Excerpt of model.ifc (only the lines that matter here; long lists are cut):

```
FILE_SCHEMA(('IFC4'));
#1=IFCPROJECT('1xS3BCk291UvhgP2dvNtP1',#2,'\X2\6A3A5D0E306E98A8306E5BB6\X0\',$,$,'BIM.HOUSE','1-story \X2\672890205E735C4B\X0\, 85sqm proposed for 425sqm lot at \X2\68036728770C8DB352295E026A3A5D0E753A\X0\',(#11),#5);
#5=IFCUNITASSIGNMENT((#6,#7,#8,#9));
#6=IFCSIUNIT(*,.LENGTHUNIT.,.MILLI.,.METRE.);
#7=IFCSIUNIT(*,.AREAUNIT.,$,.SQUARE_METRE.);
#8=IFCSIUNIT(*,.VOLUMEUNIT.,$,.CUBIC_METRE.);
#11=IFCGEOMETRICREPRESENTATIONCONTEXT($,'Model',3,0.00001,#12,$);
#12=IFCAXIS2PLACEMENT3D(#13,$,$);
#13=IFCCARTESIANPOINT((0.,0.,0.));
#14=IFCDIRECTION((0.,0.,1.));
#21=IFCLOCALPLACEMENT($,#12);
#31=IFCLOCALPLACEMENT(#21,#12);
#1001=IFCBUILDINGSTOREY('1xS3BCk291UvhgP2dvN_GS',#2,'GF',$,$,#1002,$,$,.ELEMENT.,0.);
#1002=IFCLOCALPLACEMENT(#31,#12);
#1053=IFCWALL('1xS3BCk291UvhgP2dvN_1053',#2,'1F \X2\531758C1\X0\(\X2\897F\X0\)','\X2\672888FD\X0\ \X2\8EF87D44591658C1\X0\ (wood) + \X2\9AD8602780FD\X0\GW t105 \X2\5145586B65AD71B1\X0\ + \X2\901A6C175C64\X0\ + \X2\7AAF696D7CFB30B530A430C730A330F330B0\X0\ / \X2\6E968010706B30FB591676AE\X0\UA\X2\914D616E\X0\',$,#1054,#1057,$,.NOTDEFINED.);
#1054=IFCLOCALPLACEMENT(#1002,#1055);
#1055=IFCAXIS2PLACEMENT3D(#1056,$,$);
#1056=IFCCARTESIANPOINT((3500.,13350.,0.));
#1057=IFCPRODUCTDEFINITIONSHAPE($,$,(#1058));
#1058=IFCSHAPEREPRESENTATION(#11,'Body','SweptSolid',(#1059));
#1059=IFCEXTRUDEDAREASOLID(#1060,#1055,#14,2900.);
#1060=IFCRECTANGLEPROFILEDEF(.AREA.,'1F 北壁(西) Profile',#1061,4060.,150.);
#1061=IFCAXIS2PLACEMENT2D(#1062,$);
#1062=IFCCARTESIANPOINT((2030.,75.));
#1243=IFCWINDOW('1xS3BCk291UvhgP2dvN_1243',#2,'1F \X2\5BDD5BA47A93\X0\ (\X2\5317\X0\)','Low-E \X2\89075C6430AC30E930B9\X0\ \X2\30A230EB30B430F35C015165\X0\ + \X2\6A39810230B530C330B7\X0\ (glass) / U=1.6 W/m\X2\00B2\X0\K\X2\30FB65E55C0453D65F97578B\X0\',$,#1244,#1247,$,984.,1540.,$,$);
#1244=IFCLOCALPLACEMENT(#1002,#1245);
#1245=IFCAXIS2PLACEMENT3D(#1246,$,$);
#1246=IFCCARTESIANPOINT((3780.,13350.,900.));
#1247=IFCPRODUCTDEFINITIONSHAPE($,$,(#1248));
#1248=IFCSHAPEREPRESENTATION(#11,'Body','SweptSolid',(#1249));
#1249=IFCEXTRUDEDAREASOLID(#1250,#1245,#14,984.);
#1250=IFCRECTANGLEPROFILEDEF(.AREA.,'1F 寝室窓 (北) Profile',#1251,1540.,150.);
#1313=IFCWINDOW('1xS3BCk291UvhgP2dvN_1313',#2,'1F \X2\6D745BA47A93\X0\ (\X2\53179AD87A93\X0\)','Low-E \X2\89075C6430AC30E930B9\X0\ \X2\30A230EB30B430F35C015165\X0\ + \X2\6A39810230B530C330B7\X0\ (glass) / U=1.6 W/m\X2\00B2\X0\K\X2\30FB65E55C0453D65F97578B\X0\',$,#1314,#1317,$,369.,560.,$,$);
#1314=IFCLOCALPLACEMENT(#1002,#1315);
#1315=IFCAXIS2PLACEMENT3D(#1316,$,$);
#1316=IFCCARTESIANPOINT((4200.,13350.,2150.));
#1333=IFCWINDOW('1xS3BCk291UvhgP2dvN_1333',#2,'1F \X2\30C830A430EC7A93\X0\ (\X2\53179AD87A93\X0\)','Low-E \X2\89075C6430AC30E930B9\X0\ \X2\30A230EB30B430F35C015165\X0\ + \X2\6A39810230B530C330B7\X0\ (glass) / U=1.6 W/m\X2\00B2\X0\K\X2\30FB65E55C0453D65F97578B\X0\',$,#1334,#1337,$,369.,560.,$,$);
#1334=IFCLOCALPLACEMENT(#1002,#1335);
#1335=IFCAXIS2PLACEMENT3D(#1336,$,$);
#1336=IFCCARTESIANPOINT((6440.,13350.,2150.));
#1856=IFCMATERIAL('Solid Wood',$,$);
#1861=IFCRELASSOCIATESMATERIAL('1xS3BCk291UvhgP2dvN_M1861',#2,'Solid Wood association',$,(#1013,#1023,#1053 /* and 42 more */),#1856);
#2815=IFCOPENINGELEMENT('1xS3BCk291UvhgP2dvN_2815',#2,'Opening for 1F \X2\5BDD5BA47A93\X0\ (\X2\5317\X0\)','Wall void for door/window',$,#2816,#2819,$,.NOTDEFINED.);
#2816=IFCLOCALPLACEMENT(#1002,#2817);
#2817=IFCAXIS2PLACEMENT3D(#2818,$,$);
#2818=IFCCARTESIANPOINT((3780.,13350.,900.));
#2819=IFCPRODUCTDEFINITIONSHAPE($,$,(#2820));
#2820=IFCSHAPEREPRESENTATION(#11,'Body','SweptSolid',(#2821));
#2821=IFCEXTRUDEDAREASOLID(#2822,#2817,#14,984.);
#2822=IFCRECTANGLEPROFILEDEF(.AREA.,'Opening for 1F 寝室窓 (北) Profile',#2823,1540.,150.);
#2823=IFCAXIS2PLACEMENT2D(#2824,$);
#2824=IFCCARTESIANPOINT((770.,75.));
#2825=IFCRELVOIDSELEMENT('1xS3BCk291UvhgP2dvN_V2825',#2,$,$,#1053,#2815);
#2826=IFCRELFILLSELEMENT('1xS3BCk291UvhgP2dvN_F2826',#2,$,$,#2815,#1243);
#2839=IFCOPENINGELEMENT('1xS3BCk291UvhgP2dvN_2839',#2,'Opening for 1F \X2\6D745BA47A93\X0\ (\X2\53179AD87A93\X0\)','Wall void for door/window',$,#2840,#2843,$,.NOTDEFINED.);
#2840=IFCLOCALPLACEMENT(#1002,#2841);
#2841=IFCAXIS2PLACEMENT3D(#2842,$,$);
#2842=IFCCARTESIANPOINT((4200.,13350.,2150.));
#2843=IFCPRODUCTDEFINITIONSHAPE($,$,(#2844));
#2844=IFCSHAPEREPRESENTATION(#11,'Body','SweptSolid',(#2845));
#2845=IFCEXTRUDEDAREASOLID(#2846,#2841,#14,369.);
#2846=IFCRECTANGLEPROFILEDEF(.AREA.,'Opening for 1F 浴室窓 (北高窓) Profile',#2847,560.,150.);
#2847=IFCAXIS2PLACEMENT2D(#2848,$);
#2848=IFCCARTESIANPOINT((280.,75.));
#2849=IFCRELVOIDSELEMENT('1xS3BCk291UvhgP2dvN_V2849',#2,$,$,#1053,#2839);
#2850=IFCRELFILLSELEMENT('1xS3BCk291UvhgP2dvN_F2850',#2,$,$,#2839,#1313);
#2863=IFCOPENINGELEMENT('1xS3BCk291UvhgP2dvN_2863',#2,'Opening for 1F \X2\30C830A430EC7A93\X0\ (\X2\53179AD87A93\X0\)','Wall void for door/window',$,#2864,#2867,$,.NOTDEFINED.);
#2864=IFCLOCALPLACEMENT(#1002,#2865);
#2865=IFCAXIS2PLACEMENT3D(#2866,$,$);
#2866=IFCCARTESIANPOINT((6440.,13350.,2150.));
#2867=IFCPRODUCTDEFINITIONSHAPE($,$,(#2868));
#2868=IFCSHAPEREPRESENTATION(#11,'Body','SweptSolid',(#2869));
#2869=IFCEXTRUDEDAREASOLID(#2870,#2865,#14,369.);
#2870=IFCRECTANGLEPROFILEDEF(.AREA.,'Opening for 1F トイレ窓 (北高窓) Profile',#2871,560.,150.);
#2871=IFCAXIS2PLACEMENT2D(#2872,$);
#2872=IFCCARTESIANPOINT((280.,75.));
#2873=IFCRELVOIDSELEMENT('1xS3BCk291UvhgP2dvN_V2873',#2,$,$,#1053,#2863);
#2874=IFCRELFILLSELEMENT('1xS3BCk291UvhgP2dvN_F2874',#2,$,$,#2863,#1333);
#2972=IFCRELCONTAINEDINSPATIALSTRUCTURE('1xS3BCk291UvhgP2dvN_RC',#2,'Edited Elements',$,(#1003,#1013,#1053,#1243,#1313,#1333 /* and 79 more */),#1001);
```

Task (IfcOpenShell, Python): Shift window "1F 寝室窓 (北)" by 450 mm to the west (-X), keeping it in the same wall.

```python
import ifcopenshell
import ifcopenshell.api.geometry
import ifcopenshell.util.placement

model = ifcopenshell.open("model.ifc")

window = model.by_guid("1xS3BCk291UvhgP2dvN_1243")
opening = window.FillsVoids[0].RelatingOpeningElement
wall = opening.VoidsElements[0].RelatingBuildingElement

wall_matrix = ifcopenshell.util.placement.get_local_placement(wall.ObjectPlacement)
shift = wall_matrix[:3, 0] * -450.0
before = ifcopenshell.util.placement.get_local_placement(window.ObjectPlacement)[:3, 3].copy()

# The window is not placed relative to its opening, so move both.
for product in (opening, window):
    matrix = ifcopenshell.util.placement.get_local_placement(product.ObjectPlacement)
    matrix[:3, 3] += shift
    ifcopenshell.api.geometry.edit_object_placement(model, product=product, matrix=matrix, is_si=False)

after = ifcopenshell.util.placement.get_local_placement(window.ObjectPlacement)[:3, 3]
print("window moved by", (after - before).round(3) + 0.0)

model.write("model_updated.ifc")
```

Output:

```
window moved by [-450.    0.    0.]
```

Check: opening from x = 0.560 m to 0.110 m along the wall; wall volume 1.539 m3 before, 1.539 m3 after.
